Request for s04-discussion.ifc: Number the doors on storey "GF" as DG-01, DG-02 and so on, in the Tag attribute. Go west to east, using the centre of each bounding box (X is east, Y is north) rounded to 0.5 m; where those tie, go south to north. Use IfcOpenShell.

First a look at what the model holds.

```python
import ifcopenshell
import ifcopenshell.util.element
import ifcopenshell.util.placement

model = ifcopenshell.open("s04-discussion.ifc")
print(model.schema)
storey = next(s for s in model.by_type("IfcBuildingStorey") if s.Name == "GF")
doors = [e for e in ifcopenshell.util.element.get_decomposition(storey) if e.is_a("IfcDoor")]
for e in sorted(doors, key=lambda e: e.id()):
    origin = ifcopenshell.util.placement.get_local_placement(e.ObjectPlacement)[:3, 3]
    print(e.id(), e.Tag, e.Name, origin.round(2) + 0.0, sep=" | ")
```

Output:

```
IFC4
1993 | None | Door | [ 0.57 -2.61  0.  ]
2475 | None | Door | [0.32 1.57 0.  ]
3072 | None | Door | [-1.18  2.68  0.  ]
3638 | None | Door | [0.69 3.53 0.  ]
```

```python
import ifcopenshell
import ifcopenshell.geom
import ifcopenshell.util.element
import ifcopenshell.util.shape

model = ifcopenshell.open("s04-discussion.ifc")
settings = ifcopenshell.geom.settings()
settings.set("use-world-coords", True)


def centre(element):
    shape = ifcopenshell.geom.create_shape(settings, element)
    return ifcopenshell.util.shape.get_bbox_centroid(shape.geometry)


storey = next(s for s in model.by_type("IfcBuildingStorey") if s.Name == "GF")
doors = [e for e in ifcopenshell.util.element.get_decomposition(storey) if e.is_a("IfcDoor")]

# Insertion points can sit at a corner or the storey origin, so sort by the geometry (in metres).
centres = {e: centre(e) for e in doors}
doors.sort(key=lambda e: (round(centres[e][0] / 0.5), centres[e][1]))

for i, e in enumerate(doors, start=1):
    number = f"DG-{i:02d}"
    e.Tag = number
    print(e.id(), number)

model.write("s04-discussion_edited.ifc")
```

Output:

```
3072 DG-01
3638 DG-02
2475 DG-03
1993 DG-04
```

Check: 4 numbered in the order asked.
